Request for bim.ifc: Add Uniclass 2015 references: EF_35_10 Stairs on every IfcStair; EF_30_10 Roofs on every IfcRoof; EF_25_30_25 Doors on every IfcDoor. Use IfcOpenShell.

First a look at what the model holds.

```python
import ifcopenshell

model = ifcopenshell.open("bim.ifc")
print(model.schema)
print("classifications:", [c.Name for c in model.by_type("IfcClassification")])
for ifc_class in ("IfcDoor", "IfcRoof", "IfcStair", "IfcWall", "IfcWindow"):
    print(ifc_class, len(model.by_type(ifc_class)))
```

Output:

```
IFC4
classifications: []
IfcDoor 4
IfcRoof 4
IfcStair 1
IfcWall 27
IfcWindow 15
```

```python
import ifcopenshell
import ifcopenshell.api.classification

model = ifcopenshell.open("bim.ifc")

system = ifcopenshell.api.classification.add_classification(model, classification="Uniclass 2015")

codes = {
    "IfcStair": ("EF_35_10", "Stairs"),
    "IfcRoof": ("EF_30_10", "Roofs"),
    "IfcDoor": ("EF_25_30_25", "Doors"),
}
for ifc_class, (code, name) in codes.items():
    products = model.by_type(ifc_class)
    ifcopenshell.api.classification.add_reference(
        model, products=products, classification=system, identification=code, name=name
    )
    print(code, len(products))

model.write("bim_rev.ifc")
```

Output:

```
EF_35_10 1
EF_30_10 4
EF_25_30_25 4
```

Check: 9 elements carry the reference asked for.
